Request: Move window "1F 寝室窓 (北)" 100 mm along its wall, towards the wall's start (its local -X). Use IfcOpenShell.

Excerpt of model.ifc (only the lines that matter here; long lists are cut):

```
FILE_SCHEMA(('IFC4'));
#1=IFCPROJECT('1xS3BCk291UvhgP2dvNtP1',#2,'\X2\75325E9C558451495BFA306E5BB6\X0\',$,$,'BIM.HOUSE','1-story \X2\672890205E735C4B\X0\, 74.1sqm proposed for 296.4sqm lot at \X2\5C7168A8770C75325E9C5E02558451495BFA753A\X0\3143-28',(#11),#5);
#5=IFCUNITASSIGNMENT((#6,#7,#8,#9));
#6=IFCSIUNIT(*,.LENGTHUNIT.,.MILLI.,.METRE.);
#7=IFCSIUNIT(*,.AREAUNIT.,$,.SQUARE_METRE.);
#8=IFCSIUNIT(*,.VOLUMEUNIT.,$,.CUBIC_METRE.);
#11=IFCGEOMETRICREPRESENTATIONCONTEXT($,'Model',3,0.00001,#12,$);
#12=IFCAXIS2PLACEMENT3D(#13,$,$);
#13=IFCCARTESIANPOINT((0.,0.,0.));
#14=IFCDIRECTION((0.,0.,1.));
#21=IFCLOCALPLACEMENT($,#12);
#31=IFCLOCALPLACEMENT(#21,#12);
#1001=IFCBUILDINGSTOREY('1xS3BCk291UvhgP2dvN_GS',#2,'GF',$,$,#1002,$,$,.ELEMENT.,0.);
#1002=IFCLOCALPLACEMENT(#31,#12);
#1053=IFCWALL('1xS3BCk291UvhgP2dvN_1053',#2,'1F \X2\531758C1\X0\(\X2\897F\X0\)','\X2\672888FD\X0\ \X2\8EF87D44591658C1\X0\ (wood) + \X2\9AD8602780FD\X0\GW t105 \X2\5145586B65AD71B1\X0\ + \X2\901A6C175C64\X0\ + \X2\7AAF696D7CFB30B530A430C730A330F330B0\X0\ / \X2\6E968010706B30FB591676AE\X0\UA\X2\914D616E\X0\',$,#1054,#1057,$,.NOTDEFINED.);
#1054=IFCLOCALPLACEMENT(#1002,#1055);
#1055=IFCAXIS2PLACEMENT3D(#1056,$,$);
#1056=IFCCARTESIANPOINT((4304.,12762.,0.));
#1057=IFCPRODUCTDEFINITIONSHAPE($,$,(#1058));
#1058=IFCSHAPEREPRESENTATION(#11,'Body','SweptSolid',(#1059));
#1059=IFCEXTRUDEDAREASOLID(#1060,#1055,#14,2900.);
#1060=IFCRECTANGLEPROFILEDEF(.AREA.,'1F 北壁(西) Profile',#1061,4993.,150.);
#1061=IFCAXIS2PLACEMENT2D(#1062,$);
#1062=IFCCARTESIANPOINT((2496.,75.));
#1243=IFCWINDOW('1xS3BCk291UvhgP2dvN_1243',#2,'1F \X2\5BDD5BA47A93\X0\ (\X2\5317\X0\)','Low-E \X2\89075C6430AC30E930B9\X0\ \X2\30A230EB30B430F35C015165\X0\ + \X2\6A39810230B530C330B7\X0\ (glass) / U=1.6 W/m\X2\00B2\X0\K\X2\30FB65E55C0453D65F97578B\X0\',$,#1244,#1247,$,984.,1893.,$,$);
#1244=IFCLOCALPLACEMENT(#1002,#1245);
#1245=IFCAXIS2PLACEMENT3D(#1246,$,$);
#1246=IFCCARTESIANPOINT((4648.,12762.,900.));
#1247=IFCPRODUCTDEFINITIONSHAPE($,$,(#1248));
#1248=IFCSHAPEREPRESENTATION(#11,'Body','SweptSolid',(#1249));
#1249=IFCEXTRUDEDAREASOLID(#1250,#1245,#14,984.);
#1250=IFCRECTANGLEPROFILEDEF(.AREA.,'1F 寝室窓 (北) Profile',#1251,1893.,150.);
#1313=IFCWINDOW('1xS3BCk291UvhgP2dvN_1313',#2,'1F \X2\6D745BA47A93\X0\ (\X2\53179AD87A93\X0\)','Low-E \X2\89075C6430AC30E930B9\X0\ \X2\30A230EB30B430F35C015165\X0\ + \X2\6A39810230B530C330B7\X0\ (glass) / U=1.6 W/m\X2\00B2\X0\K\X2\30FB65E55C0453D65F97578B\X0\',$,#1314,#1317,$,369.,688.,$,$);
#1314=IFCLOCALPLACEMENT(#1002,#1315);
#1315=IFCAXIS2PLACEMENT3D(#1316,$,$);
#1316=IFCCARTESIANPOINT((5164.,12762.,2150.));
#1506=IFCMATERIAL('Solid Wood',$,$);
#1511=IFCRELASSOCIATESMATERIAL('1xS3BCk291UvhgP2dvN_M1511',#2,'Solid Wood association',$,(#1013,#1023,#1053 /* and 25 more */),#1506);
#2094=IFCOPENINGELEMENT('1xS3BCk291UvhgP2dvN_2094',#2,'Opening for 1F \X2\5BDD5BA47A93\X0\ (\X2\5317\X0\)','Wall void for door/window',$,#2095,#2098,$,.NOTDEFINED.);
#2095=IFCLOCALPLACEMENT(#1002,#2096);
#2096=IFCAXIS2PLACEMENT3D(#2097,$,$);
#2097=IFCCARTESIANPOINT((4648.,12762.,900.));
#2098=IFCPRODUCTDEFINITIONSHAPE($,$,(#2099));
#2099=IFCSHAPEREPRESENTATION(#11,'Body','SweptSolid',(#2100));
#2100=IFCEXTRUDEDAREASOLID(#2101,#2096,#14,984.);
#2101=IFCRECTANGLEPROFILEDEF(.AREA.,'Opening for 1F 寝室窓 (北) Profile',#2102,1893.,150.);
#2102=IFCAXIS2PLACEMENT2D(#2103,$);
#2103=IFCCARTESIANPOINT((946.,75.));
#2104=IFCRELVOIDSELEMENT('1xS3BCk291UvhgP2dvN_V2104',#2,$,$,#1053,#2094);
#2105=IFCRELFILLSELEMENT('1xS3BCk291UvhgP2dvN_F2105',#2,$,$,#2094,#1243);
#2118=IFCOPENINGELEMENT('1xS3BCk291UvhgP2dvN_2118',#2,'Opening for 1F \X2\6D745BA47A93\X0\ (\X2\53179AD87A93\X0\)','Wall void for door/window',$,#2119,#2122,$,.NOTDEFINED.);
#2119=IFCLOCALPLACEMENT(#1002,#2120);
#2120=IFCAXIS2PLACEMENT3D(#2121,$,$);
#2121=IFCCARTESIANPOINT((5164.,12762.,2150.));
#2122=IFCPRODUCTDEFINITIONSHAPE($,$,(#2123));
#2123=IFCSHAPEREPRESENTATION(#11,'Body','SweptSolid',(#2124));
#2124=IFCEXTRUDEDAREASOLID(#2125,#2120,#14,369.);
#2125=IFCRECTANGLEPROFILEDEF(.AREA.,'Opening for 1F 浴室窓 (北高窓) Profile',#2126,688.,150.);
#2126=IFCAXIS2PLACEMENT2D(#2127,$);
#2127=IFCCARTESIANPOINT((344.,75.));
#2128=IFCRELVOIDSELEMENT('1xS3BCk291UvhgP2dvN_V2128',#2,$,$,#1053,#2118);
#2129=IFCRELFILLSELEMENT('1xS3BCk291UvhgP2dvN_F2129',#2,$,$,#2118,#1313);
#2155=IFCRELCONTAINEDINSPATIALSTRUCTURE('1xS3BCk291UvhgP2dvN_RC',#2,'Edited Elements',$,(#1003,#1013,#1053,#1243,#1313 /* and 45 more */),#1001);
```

```python
import ifcopenshell
import ifcopenshell.api.geometry
import ifcopenshell.util.placement

model = ifcopenshell.open("model.ifc")

window = model.by_guid("1xS3BCk291UvhgP2dvN_1243")
opening = window.FillsVoids[0].RelatingOpeningElement
wall = opening.VoidsElements[0].RelatingBuildingElement

wall_matrix = ifcopenshell.util.placement.get_local_placement(wall.ObjectPlacement)
shift = wall_matrix[:3, 0] * -100.0
before = ifcopenshell.util.placement.get_local_placement(window.ObjectPlacement)[:3, 3].copy()

# The window is not placed relative to its opening, so move both.
for product in (opening, window):
    matrix = ifcopenshell.util.placement.get_local_placement(product.ObjectPlacement)
    matrix[:3, 3] += shift
    ifcopenshell.api.geometry.edit_object_placement(model, product=product, matrix=matrix, is_si=False)

after = ifcopenshell.util.placement.get_local_placement(window.ObjectPlacement)[:3, 3]
print("window moved by", (after - before).round(3) + 0.0)

model.write("model_v2.ifc")
```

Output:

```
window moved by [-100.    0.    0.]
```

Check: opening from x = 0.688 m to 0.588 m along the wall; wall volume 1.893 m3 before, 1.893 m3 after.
